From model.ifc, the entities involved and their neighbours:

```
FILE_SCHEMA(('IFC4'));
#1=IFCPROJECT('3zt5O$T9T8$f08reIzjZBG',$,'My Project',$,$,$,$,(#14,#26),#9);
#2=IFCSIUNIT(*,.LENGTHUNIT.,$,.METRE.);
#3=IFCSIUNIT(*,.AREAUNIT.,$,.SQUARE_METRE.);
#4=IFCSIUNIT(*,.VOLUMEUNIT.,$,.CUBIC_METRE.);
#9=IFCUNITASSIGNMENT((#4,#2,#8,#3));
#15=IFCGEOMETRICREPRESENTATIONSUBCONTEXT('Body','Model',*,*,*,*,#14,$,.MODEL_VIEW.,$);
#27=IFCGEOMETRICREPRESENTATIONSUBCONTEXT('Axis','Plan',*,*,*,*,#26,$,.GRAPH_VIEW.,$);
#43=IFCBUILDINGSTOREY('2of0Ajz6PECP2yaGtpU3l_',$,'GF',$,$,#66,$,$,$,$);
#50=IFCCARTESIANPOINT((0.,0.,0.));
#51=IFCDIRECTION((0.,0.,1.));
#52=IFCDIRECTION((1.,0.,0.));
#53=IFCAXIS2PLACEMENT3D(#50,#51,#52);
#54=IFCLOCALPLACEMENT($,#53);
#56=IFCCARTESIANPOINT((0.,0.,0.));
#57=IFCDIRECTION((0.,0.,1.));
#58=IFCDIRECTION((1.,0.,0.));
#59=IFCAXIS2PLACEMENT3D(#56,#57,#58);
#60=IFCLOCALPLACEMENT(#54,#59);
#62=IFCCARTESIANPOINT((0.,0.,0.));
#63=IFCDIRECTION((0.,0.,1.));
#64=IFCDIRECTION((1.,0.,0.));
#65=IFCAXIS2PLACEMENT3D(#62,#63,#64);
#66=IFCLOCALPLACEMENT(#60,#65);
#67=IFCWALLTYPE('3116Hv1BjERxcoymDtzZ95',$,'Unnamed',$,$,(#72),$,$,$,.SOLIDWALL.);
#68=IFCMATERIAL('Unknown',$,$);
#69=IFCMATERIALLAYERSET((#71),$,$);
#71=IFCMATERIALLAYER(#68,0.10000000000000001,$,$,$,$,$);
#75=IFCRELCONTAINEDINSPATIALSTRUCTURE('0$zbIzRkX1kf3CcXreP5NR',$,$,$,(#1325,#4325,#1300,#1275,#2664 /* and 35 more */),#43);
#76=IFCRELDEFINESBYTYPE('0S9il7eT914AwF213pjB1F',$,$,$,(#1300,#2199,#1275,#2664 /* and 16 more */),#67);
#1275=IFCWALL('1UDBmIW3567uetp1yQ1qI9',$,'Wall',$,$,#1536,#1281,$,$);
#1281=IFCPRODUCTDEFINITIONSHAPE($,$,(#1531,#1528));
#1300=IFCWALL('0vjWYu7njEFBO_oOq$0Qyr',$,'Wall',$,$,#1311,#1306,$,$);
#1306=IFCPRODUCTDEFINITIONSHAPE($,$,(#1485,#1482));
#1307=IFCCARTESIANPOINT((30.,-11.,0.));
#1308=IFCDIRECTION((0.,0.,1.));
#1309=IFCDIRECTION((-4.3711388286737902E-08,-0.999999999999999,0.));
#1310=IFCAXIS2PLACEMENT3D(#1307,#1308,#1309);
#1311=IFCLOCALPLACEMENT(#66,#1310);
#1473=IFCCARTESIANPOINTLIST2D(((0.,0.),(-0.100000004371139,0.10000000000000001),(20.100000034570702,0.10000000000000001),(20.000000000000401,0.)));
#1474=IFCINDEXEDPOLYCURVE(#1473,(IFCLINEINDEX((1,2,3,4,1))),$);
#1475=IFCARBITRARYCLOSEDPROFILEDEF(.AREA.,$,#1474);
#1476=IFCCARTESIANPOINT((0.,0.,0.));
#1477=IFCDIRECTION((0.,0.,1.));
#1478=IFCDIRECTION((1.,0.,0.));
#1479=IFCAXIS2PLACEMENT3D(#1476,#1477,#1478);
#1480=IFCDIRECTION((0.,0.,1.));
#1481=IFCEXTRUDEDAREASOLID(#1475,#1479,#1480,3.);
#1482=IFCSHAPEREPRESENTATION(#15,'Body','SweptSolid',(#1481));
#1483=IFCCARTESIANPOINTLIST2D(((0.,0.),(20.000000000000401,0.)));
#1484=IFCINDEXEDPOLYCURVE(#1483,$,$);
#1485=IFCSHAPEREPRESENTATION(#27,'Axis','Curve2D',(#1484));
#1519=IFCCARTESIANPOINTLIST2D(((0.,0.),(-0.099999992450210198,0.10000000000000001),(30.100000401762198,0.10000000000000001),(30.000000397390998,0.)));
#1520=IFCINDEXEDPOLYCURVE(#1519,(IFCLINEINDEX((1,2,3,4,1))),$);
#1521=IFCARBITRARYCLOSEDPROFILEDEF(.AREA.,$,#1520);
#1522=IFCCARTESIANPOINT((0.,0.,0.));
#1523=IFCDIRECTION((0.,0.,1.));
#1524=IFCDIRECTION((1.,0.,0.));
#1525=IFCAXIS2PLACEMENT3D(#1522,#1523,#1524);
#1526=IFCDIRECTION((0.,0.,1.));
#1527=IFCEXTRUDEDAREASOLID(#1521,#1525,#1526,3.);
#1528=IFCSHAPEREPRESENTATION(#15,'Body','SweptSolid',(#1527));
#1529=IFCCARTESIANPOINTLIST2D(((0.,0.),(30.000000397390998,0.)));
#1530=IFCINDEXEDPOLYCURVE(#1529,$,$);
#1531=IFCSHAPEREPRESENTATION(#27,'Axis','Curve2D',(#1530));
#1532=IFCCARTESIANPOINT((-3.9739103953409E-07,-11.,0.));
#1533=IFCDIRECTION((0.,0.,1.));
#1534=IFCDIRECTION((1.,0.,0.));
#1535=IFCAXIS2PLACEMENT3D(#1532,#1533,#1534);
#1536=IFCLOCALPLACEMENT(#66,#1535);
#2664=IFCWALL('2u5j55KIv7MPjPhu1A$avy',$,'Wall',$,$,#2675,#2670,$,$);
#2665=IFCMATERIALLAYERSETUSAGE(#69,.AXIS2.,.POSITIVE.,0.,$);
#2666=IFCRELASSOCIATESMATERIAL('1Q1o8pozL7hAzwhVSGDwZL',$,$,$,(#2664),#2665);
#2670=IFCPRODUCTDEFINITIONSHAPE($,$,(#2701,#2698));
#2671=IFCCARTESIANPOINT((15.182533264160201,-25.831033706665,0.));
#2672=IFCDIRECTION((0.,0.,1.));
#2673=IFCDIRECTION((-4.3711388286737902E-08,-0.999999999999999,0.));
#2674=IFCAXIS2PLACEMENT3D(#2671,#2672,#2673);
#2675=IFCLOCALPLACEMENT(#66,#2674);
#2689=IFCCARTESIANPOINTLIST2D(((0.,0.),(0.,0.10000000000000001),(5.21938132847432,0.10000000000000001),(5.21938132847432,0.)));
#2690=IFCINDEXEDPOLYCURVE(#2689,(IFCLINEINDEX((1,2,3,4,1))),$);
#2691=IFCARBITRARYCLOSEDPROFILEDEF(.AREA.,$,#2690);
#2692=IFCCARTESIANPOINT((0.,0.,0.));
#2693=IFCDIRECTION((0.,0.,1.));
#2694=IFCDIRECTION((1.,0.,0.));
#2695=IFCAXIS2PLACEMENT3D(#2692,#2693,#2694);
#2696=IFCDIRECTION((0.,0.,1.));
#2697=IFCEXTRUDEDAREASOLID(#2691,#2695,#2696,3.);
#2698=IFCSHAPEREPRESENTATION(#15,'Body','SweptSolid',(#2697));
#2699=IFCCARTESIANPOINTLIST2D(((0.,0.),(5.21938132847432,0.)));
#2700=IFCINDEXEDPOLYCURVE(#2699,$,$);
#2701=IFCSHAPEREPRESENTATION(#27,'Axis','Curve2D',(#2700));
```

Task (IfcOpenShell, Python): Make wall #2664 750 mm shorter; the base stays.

```python
import ifcopenshell
import ifcopenshell.geom
import ifcopenshell.util.representation
import ifcopenshell.util.shape
import ifcopenshell.util.unit

model = ifcopenshell.open("model.ifc")
unit_scale = ifcopenshell.util.unit.calculate_unit_scale(model)
settings = ifcopenshell.geom.settings()


def volume(element):
    """Net volume in cubic metres, openings subtracted."""
    shape = ifcopenshell.geom.create_shape(settings, element)
    return ifcopenshell.util.shape.get_volume(shape.geometry)


wall = model.by_guid("2u5j55KIv7MPjPhu1A$avy")
before = volume(wall)

body = ifcopenshell.util.representation.get_representation(wall, "Model", "Body")
solid = body.Items[0]
old_height = solid.Depth
solid.Depth -= 0.75 / unit_scale
after = volume(wall)

print(f"height {old_height:g} -> {solid.Depth:g}, volume {before:.3f} -> {after:.3f} m3")

model.write("model-out.ifc")
```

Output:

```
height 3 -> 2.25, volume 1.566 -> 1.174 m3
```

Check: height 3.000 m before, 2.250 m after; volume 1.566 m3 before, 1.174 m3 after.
